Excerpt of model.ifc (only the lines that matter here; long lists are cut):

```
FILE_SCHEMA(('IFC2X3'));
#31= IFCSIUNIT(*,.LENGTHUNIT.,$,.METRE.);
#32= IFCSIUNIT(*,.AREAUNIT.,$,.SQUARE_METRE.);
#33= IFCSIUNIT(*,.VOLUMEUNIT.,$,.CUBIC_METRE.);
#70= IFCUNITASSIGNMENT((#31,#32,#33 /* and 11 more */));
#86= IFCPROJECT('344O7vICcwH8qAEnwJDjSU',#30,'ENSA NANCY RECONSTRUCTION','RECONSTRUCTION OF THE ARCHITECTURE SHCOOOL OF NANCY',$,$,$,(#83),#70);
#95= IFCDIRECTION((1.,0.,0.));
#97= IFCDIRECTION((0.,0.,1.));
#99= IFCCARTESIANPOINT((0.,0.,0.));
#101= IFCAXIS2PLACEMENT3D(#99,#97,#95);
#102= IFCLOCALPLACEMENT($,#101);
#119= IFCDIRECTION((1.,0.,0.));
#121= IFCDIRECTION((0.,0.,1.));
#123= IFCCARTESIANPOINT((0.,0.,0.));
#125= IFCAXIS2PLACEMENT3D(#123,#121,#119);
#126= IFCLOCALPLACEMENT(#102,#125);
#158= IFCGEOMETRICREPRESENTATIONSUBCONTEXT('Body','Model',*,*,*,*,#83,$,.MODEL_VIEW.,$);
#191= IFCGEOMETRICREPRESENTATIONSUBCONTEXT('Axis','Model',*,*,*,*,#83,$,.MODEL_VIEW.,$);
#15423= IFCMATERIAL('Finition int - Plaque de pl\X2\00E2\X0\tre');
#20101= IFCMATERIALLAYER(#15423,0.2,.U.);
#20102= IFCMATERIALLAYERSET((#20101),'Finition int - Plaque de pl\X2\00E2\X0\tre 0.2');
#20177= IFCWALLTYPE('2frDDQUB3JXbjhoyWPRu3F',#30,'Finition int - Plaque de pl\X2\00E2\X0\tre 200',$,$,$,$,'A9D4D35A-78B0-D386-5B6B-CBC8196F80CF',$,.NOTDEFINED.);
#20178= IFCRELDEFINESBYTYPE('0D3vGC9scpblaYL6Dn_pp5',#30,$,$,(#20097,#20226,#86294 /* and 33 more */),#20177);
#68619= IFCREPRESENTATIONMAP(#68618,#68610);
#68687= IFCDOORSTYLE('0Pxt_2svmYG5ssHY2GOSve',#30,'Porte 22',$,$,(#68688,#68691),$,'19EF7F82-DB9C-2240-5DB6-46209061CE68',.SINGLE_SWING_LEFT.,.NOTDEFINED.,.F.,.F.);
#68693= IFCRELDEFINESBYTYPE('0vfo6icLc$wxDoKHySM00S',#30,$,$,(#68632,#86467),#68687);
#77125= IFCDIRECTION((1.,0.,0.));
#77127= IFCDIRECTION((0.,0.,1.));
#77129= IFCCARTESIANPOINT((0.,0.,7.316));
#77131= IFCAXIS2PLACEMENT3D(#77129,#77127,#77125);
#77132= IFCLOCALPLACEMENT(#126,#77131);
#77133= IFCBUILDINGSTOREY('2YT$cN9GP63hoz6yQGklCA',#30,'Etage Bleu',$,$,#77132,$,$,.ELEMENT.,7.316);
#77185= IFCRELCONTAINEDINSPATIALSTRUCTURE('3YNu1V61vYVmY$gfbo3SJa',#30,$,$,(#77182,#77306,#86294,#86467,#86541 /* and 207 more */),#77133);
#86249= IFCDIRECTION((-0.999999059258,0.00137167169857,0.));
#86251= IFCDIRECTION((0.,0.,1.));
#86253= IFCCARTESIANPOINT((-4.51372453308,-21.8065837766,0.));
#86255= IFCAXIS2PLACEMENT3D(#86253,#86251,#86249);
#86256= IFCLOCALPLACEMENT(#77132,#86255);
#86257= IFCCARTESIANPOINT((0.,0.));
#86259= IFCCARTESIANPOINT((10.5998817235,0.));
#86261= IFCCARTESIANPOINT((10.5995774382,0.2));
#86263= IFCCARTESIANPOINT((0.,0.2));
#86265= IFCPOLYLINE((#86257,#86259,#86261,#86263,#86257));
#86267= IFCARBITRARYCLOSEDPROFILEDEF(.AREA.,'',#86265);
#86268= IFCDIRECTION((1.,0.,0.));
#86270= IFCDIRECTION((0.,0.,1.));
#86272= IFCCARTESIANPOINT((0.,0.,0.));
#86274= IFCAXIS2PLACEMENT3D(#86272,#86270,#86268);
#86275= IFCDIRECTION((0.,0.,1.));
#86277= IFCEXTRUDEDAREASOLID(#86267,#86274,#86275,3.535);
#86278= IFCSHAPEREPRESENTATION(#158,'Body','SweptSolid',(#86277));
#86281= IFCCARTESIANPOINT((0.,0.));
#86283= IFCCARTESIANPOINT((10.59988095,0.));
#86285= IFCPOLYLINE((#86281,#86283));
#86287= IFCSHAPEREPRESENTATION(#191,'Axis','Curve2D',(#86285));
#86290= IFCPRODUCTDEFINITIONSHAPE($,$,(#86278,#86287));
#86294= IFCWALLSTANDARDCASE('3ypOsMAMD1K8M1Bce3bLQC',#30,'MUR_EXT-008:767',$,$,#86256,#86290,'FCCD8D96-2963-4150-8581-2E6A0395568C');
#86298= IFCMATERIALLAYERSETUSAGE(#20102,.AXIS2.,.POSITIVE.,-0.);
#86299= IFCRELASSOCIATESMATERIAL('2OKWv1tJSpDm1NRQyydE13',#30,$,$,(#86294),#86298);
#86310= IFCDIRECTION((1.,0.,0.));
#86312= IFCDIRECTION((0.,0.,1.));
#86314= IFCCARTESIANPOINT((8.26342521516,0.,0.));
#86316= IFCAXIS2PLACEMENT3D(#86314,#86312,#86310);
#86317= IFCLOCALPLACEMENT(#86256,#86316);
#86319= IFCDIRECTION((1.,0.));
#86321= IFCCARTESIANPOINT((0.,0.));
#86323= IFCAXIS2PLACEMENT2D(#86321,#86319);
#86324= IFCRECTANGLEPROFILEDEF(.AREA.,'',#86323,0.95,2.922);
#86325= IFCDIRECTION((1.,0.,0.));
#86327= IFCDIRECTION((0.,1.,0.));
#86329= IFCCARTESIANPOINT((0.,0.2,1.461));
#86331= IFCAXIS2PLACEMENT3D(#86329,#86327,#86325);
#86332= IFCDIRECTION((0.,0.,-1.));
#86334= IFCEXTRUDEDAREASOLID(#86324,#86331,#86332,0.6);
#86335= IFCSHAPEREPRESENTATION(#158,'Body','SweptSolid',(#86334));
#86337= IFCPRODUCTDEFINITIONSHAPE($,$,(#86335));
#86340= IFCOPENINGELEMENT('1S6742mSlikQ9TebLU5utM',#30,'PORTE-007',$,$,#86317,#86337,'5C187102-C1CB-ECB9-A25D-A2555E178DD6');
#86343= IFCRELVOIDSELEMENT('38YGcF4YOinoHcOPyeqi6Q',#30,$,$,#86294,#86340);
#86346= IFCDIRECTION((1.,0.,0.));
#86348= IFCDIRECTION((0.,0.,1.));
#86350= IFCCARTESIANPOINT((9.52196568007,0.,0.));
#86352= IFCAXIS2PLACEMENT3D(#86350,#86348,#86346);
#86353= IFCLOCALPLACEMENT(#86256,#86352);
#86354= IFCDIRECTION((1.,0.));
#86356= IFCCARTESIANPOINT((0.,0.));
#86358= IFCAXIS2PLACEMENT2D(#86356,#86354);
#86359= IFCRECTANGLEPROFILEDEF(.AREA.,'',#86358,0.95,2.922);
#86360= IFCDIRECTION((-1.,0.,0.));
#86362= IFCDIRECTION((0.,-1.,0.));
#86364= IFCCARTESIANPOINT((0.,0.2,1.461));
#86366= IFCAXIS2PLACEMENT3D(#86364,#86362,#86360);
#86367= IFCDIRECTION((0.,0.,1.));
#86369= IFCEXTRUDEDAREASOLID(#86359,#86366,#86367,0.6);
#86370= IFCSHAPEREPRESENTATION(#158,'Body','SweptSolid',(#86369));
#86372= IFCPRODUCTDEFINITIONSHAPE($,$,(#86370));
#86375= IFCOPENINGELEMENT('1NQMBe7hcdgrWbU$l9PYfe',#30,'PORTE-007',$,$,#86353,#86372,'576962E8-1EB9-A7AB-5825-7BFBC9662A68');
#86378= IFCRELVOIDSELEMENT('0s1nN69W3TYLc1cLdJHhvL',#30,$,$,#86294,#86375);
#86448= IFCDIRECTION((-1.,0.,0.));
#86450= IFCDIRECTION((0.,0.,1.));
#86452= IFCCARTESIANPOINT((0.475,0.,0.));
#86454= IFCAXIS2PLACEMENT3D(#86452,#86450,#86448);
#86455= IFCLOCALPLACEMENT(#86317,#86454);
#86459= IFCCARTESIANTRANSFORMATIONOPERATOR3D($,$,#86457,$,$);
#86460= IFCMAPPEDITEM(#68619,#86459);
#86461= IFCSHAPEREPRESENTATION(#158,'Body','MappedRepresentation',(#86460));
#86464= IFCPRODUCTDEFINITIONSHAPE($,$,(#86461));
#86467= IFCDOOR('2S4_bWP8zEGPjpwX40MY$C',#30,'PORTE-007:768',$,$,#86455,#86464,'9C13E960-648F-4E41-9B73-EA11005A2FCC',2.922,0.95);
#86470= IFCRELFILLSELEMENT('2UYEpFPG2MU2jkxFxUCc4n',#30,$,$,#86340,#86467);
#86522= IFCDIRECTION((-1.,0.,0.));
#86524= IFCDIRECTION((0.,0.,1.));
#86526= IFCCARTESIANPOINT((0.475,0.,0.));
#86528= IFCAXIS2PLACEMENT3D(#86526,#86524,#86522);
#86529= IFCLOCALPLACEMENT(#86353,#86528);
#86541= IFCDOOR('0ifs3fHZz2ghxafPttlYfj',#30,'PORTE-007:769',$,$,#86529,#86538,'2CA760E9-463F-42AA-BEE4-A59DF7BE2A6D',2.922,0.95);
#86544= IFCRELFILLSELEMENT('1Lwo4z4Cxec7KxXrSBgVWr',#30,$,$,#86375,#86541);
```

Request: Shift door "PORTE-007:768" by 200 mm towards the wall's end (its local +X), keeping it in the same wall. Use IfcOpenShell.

```python
import ifcopenshell
import ifcopenshell.api.geometry
import ifcopenshell.util.placement
import ifcopenshell.util.unit

model = ifcopenshell.open("model.ifc")
unit_scale = ifcopenshell.util.unit.calculate_unit_scale(model)

door = model.by_guid("2S4_bWP8zEGPjpwX40MY$C")
opening = door.FillsVoids[0].RelatingOpeningElement
wall = opening.VoidsElements[0].RelatingBuildingElement

wall_matrix = ifcopenshell.util.placement.get_local_placement(wall.ObjectPlacement)
shift = wall_matrix[:3, 0] * 0.2 / unit_scale
before = ifcopenshell.util.placement.get_local_placement(door.ObjectPlacement)[:3, 3].copy()

# The door is placed relative to its opening, so it follows when the opening moves.
matrix = ifcopenshell.util.placement.get_local_placement(opening.ObjectPlacement)
matrix[:3, 3] += shift
ifcopenshell.api.geometry.edit_object_placement(
    model, product=opening, matrix=matrix, is_si=False, should_transform_children=True
)

after = ifcopenshell.util.placement.get_local_placement(door.ObjectPlacement)[:3, 3]
print("door moved by", (after - before).round(3) + 0.0)

model.write("model-out.ifc")
```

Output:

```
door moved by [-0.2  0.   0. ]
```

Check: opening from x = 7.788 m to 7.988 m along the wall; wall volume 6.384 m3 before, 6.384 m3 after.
